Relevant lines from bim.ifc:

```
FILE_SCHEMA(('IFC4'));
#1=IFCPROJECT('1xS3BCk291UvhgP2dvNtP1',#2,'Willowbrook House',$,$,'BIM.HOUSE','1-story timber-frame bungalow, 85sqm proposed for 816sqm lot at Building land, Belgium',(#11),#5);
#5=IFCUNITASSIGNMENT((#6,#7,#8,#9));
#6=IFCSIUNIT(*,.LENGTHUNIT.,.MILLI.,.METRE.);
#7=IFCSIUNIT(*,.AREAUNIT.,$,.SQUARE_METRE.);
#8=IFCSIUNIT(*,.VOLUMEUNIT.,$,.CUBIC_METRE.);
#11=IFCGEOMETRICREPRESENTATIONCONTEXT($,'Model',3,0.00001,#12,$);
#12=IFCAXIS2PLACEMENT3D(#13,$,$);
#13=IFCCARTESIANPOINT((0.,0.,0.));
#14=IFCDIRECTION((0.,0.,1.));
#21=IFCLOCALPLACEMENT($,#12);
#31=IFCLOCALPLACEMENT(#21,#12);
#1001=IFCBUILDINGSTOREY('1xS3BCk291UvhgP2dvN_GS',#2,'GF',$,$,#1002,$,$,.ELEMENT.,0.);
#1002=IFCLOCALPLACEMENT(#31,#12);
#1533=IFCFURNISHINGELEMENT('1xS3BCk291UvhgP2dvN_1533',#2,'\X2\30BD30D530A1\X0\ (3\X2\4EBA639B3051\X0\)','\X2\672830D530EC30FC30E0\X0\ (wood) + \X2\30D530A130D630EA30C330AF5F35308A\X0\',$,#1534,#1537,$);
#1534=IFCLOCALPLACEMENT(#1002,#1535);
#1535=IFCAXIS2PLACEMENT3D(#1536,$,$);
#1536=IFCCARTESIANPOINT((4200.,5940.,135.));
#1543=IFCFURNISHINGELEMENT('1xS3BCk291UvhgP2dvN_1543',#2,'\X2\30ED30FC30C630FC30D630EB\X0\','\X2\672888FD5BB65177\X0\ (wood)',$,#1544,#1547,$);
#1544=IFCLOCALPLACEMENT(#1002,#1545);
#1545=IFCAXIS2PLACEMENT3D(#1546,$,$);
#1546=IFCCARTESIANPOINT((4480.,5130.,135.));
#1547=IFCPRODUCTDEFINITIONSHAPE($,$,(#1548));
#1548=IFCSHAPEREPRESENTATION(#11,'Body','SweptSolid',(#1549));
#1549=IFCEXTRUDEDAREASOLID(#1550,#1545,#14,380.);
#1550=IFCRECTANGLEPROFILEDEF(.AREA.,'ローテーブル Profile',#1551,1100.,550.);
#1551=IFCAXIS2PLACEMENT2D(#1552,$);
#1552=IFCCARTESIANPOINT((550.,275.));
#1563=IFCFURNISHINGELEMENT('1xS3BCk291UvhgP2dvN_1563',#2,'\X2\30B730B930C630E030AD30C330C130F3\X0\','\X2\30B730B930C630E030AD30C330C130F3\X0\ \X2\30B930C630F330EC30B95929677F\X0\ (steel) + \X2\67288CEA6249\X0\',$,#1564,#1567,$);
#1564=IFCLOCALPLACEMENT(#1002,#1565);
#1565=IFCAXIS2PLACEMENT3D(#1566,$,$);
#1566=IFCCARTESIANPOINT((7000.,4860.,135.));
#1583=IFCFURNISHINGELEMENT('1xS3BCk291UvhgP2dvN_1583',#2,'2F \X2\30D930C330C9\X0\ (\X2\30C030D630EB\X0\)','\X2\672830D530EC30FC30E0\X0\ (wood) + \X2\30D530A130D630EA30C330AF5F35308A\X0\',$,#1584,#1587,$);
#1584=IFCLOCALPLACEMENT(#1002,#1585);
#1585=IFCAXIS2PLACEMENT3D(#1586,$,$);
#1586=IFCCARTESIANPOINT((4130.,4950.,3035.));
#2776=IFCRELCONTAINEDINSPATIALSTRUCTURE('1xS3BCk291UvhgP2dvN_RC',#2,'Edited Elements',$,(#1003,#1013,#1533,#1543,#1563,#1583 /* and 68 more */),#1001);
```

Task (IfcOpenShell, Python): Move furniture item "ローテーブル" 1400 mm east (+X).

```python
import ifcopenshell
import ifcopenshell.api.geometry
import ifcopenshell.util.placement
import ifcopenshell.util.unit

model = ifcopenshell.open("bim.ifc")
unit_scale = ifcopenshell.util.unit.calculate_unit_scale(model)

item = model.by_guid("1xS3BCk291UvhgP2dvN_1543")
matrix = ifcopenshell.util.placement.get_local_placement(item.ObjectPlacement)
matrix[0, 3] += 1.4 / unit_scale
ifcopenshell.api.geometry.edit_object_placement(model, product=item, matrix=matrix, is_si=False)

print(ifcopenshell.util.placement.get_local_placement(item.ObjectPlacement).round(3) + 0.0)

model.write("bim_rev.ifc")
```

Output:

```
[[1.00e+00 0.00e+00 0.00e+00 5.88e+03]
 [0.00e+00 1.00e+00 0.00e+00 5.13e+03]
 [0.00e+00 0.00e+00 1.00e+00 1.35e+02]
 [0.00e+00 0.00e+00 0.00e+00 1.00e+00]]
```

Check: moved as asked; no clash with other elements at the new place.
